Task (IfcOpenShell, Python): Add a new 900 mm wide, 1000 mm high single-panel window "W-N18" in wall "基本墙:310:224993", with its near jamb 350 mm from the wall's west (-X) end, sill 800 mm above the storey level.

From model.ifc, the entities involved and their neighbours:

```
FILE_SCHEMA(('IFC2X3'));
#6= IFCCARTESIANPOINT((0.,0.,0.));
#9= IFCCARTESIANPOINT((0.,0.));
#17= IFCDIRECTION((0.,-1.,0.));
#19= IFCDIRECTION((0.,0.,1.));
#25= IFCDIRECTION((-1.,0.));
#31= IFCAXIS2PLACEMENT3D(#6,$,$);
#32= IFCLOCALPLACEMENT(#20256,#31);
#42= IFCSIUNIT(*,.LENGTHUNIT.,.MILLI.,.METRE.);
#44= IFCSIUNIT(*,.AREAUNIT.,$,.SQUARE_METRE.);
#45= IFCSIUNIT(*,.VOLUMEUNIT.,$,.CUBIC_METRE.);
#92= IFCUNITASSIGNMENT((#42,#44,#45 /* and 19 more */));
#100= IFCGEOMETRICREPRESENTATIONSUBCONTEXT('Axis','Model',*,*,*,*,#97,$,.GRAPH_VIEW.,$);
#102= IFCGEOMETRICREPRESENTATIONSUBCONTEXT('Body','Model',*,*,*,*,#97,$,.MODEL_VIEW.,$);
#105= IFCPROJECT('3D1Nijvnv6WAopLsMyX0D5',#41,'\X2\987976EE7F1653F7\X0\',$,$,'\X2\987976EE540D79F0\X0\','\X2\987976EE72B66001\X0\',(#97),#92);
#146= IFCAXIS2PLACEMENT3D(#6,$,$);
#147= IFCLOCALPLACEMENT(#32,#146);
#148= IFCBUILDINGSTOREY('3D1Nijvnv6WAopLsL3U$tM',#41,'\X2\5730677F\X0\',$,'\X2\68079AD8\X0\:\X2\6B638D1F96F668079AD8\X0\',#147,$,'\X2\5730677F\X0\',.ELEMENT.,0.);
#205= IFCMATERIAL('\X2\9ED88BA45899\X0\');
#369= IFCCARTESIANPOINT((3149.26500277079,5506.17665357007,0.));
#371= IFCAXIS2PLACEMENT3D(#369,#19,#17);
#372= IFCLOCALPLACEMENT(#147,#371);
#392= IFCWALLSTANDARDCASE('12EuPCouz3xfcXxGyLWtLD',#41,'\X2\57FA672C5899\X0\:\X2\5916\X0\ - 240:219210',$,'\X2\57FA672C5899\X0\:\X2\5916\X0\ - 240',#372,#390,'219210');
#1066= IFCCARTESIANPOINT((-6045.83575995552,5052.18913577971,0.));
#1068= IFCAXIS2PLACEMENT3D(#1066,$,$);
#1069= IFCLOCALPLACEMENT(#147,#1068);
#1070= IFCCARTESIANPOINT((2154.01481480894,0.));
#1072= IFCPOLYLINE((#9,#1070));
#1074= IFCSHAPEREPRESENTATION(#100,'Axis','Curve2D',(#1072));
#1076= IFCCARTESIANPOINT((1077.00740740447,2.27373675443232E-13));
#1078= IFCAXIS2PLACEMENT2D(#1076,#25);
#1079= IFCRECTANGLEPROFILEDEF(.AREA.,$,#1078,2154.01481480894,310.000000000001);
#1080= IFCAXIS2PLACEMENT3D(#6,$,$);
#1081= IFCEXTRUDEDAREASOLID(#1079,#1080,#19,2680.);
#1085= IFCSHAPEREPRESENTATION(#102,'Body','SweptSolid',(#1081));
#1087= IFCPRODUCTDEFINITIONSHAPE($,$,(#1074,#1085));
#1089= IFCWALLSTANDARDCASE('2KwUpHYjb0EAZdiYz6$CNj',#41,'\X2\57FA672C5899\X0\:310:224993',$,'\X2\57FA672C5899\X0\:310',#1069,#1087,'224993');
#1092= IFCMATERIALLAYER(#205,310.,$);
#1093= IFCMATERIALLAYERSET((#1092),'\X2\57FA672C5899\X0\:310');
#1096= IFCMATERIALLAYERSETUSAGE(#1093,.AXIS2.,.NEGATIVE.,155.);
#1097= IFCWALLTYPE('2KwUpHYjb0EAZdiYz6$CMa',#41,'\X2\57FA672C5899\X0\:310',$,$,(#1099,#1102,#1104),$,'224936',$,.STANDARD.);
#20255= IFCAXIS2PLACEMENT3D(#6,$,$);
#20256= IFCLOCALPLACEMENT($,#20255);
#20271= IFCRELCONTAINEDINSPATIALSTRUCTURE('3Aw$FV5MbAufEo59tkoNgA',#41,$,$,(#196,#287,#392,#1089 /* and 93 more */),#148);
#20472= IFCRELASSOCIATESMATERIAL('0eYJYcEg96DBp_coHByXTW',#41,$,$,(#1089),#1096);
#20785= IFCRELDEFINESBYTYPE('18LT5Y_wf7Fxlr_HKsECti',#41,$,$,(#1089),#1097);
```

```python
import numpy as np
import ifcopenshell
import ifcopenshell.api.feature
import ifcopenshell.api.geometry
import ifcopenshell.api.root
import ifcopenshell.api.spatial
import ifcopenshell.api.type
import ifcopenshell.geom
import ifcopenshell.util.element
import ifcopenshell.util.placement
import ifcopenshell.util.representation
import ifcopenshell.util.shape
import ifcopenshell.util.unit

model = ifcopenshell.open("model.ifc")
unit_scale = ifcopenshell.util.unit.calculate_unit_scale(model)
settings = ifcopenshell.geom.settings()


def volume(element):
    """Net volume in cubic metres, openings subtracted."""
    shape = ifcopenshell.geom.create_shape(settings, element)
    return ifcopenshell.util.shape.get_volume(shape.geometry)


wall = model.by_id(1089)
storey = ifcopenshell.util.element.get_container(wall, ifc_class="IfcBuildingStorey")
context = ifcopenshell.util.representation.get_context(model, "Model", "Body", "MODEL_VIEW")
before = volume(wall)

width, height, from_end, sill = 0.9, 1, 0.35, 0.8  # metres

# The wall runs along its own X axis, and the end named is its -X end.
wall_shape = ifcopenshell.geom.create_shape(settings, wall)
x, y, z = ifcopenshell.util.shape.get_vertices(wall_shape.geometry).T
start = x.min() + from_end
face, thickness = float(y.min()), float(y.max() - y.min())
wall_matrix = ifcopenshell.util.placement.get_local_placement(wall.ObjectPlacement)
level = ifcopenshell.util.placement.get_local_placement(storey.ObjectPlacement)[2, 3]


def in_wall(x, y):
    """Placement at x, y metres in the wall's axes, at sill height."""
    matrix = wall_matrix.copy()
    matrix[:, 3] = wall_matrix @ np.array([x / unit_scale, y / unit_scale, 0.0, 1.0])
    matrix[2, 3] = level + sill / unit_scale
    return matrix


# Opening: a box that overshoots both wall faces by 50 mm.
opening = ifcopenshell.api.root.create_entity(model, ifc_class="IfcOpeningElement")
box = ifcopenshell.api.geometry.add_wall_representation(
    model, context=context, length=width, height=height, thickness=thickness + 0.1
)
ifcopenshell.api.geometry.assign_representation(model, product=opening, representation=box)
ifcopenshell.api.geometry.edit_object_placement(model, product=opening, matrix=in_wall(start, face - 0.05), is_si=False)
ifcopenshell.api.feature.add_feature(model, feature=opening, element=wall)

window = ifcopenshell.api.root.create_entity(model, ifc_class="IfcWindow", name="W-N18")
window.OverallWidth, window.OverallHeight = width / unit_scale, height / unit_scale
body = ifcopenshell.api.geometry.add_window_representation(
    model,
    context=context,
    overall_width=window.OverallWidth,
    overall_height=window.OverallHeight,
    partition_type="SINGLE_PANEL",
)
ifcopenshell.api.geometry.assign_representation(model, product=window, representation=body)
ifcopenshell.api.spatial.assign_container(model, products=[window], relating_structure=storey)
fills = ifcopenshell.api.feature.add_filling(model, opening=opening, element=window)
fills.OwnerHistory = window.OwnerHistory  # required in IFC2X3

# IFC2X3 keeps the operation on the window style.
style = ifcopenshell.api.root.create_entity(model, ifc_class="IfcWindowStyle", name="W-N18")
style.OperationType, style.ConstructionType = "SINGLE_PANEL", "NOTDEFINED"
style.ParameterTakesPrecedence = style.Sizeable = False
ifcopenshell.api.type.assign_type(model, related_objects=[window], relating_type=style)

# Centre the window in the wall's thickness.
ifcopenshell.api.geometry.edit_object_placement(model, product=window, matrix=in_wall(start, face), is_si=False)
window_shape = ifcopenshell.geom.create_shape(settings, window)
depth = ifcopenshell.util.shape.get_vertices(window_shape.geometry)[:, 1]
offset = face + thickness / 2 - (depth.min() + depth.max()) / 2
ifcopenshell.api.geometry.edit_object_placement(model, product=window, matrix=in_wall(start, offset), is_si=False)

after = volume(wall)

print(f"wall volume {before:.3f} -> {after:.3f} m3")

model.write("model_updated.ifc")
```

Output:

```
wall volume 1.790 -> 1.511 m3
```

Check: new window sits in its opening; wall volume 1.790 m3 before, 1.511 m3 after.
